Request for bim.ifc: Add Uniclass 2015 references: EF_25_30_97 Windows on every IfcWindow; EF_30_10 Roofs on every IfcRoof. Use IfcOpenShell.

First a look at what the model holds.

```python
import ifcopenshell

model = ifcopenshell.open("bim.ifc")
print(model.schema)
print("classifications:", [c.Name for c in model.by_type("IfcClassification")])
for ifc_class in ("IfcDoor", "IfcRoof", "IfcStair", "IfcWall", "IfcWindow"):
    print(ifc_class, len(model.by_type(ifc_class)))
```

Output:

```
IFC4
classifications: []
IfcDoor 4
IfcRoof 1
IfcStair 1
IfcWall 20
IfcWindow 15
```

```python
import ifcopenshell
import ifcopenshell.api.classification

model = ifcopenshell.open("bim.ifc")

system = ifcopenshell.api.classification.add_classification(model, classification="Uniclass 2015")

codes = {
    "IfcWindow": ("EF_25_30_97", "Windows"),
    "IfcRoof": ("EF_30_10", "Roofs"),
}
for ifc_class, (code, name) in codes.items():
    products = model.by_type(ifc_class)
    ifcopenshell.api.classification.add_reference(
        model, products=products, classification=system, identification=code, name=name
    )
    print(code, len(products))

model.write("bim_rev.ifc")
```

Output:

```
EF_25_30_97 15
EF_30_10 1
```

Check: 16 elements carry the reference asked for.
